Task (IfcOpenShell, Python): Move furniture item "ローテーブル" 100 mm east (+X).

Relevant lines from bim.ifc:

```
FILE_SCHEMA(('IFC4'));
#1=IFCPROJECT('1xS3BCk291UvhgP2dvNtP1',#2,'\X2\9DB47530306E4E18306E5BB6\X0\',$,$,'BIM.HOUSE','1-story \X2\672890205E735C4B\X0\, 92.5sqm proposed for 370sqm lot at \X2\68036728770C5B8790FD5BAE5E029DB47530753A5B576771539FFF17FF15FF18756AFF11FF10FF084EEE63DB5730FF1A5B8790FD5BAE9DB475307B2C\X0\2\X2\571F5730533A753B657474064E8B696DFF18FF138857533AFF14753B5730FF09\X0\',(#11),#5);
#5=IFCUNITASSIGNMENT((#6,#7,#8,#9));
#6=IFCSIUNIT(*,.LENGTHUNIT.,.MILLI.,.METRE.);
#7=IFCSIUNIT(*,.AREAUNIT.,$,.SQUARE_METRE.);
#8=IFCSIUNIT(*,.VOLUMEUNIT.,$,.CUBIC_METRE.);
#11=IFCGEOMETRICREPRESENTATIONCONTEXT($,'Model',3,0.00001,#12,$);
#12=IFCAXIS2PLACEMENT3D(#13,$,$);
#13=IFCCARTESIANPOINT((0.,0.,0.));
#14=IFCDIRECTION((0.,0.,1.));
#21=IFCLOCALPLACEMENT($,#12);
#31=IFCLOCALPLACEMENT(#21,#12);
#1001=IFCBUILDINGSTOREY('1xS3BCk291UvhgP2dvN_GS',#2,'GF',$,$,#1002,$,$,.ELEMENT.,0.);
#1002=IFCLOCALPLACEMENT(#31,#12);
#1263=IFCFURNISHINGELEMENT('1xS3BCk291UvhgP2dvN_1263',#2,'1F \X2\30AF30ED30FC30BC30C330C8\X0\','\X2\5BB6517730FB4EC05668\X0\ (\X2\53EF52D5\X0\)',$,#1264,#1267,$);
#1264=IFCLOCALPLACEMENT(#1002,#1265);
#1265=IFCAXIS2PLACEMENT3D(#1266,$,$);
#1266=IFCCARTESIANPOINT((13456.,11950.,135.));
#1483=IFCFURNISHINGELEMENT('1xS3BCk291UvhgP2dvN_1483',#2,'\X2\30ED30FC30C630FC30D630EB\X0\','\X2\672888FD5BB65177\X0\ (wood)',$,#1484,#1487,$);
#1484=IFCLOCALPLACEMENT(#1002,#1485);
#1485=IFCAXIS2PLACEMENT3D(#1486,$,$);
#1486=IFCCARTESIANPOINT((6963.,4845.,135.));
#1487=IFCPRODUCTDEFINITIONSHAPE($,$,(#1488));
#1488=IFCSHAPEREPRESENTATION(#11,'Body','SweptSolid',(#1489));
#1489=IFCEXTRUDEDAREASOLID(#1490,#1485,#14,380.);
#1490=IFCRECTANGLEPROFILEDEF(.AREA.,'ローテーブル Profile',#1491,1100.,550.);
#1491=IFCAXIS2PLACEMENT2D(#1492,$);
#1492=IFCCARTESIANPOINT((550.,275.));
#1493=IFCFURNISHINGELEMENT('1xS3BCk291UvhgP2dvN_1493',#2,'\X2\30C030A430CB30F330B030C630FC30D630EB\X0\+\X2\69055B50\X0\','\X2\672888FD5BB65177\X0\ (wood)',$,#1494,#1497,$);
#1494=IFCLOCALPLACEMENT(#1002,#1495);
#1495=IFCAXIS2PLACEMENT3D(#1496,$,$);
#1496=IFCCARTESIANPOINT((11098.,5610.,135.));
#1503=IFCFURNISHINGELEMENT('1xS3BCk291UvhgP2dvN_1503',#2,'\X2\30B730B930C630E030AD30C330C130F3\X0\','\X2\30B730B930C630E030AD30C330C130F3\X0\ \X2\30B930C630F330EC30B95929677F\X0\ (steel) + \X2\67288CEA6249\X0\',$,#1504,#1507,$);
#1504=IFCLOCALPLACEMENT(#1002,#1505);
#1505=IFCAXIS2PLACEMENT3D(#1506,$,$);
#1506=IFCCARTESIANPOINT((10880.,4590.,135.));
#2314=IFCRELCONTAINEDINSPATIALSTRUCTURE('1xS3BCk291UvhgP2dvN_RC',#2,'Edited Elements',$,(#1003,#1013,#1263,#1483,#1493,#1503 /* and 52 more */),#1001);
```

```python
import ifcopenshell
import ifcopenshell.api.geometry
import ifcopenshell.util.placement
import ifcopenshell.util.unit

model = ifcopenshell.open("bim.ifc")
unit_scale = ifcopenshell.util.unit.calculate_unit_scale(model)

item = model.by_guid("1xS3BCk291UvhgP2dvN_1483")
matrix = ifcopenshell.util.placement.get_local_placement(item.ObjectPlacement)
matrix[0, 3] += 0.1 / unit_scale
ifcopenshell.api.geometry.edit_object_placement(model, product=item, matrix=matrix, is_si=False)

print(ifcopenshell.util.placement.get_local_placement(item.ObjectPlacement).round(3) + 0.0)

model.write("bim_updated.ifc")
```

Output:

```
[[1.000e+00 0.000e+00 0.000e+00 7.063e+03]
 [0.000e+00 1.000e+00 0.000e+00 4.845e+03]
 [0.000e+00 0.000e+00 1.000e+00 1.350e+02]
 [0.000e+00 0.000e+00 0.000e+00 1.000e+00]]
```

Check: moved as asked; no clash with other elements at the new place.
